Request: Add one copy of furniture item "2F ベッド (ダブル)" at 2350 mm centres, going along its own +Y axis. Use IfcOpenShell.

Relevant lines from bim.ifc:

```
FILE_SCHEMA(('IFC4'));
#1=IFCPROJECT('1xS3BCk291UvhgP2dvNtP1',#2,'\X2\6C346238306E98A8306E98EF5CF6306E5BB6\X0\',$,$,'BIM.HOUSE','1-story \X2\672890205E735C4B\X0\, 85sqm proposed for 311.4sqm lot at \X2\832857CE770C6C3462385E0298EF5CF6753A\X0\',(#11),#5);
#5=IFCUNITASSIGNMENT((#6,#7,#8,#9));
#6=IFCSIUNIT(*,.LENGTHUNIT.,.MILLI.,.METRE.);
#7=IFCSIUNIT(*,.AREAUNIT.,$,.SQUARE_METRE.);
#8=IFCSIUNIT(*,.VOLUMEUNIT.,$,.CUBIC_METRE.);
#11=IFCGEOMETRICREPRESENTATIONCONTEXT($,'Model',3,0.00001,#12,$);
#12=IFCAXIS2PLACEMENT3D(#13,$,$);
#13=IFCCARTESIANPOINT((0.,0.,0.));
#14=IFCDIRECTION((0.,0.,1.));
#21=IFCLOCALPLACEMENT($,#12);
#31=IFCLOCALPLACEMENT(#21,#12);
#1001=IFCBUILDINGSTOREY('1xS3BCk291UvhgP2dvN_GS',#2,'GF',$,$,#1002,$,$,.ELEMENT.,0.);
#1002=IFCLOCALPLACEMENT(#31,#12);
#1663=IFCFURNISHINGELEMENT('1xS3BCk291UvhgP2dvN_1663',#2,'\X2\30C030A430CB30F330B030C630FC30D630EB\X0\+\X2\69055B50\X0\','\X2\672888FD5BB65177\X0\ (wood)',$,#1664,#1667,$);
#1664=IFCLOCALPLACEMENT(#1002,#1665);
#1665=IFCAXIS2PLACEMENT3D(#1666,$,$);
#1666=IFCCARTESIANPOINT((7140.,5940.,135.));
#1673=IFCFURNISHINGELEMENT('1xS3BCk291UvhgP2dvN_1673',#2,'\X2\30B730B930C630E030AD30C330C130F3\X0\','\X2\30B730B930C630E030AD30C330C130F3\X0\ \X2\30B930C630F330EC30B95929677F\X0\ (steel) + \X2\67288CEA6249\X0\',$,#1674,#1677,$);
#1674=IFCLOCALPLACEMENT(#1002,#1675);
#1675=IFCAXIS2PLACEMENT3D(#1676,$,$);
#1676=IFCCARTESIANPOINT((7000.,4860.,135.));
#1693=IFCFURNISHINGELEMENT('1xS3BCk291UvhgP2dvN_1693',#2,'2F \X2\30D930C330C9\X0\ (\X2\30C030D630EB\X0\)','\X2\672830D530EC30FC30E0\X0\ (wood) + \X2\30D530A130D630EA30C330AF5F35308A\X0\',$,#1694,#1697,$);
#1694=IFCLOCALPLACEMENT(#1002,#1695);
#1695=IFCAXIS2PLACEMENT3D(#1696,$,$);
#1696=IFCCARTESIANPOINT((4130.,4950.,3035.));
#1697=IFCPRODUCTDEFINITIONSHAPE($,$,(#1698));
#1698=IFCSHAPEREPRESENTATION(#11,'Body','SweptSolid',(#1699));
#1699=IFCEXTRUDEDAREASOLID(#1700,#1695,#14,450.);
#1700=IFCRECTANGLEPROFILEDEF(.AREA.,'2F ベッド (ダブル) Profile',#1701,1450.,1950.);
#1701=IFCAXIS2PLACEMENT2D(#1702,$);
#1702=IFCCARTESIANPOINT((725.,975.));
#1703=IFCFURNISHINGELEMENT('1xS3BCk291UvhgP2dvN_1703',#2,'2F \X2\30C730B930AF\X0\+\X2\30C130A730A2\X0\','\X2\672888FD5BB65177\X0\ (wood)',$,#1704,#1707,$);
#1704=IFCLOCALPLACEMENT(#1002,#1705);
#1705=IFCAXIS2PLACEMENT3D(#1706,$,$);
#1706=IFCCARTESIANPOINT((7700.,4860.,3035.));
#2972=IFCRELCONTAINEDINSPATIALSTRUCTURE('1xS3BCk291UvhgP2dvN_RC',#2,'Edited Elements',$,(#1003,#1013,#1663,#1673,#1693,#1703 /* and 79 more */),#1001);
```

```python
import ifcopenshell
import ifcopenshell.api.geometry
import ifcopenshell.api.root
import ifcopenshell.util.element
import ifcopenshell.util.placement
import ifcopenshell.util.unit

model = ifcopenshell.open("bim.ifc")
unit_scale = ifcopenshell.util.unit.calculate_unit_scale(model)


def reuse_history(source, copy):
    """copy_class also copies each property set's owner history, people and application; keep the originals."""
    for rel in copy.IsDefinedBy:
        if rel.is_a("IfcRelDefinesByProperties") and (history := rel.RelatingPropertyDefinition.OwnerHistory):
            rel.RelatingPropertyDefinition.OwnerHistory = source.OwnerHistory
            ifcopenshell.util.element.remove_deep2(model, history)


source = model.by_guid("1xS3BCk291UvhgP2dvN_1693")
base = ifcopenshell.util.placement.get_local_placement(source.ObjectPlacement)
step = base[:3, 1] * 2.35 / unit_scale

for i in range(1, 2):
    copy = ifcopenshell.api.root.copy_class(model, product=source)
    copy.Representation = ifcopenshell.util.element.copy_deep(
        model, source.Representation, exclude=["IfcGeometricRepresentationContext", "IfcRepresentationMap"]
    )
    reuse_history(source, copy)
    matrix = base.copy()
    matrix[:3, 3] += i * step
    print("added at", matrix[:3, 3].round(3) + 0.0)
    ifcopenshell.api.geometry.edit_object_placement(model, product=copy, matrix=matrix, is_si=False)

model.write("bim_rev.ifc")
```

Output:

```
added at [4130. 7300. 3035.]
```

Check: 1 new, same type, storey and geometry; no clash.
